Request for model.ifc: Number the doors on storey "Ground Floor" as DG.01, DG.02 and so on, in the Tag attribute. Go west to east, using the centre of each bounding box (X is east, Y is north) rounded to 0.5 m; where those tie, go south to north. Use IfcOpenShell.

First a look at what the model holds.

```python
import ifcopenshell
import ifcopenshell.util.element
import ifcopenshell.util.placement

model = ifcopenshell.open("model.ifc")
print(model.schema)
storey = next(s for s in model.by_type("IfcBuildingStorey") if s.Name == "Ground Floor")
doors = [e for e in ifcopenshell.util.element.get_decomposition(storey) if e.is_a("IfcDoor")]
for e in sorted(doors, key=lambda e: e.id()):
    origin = ifcopenshell.util.placement.get_local_placement(e.ObjectPlacement)[:3, 3]
    print(e.id(), e.Tag, e.Name, origin.round(2) + 0.0, sep=" | ")
```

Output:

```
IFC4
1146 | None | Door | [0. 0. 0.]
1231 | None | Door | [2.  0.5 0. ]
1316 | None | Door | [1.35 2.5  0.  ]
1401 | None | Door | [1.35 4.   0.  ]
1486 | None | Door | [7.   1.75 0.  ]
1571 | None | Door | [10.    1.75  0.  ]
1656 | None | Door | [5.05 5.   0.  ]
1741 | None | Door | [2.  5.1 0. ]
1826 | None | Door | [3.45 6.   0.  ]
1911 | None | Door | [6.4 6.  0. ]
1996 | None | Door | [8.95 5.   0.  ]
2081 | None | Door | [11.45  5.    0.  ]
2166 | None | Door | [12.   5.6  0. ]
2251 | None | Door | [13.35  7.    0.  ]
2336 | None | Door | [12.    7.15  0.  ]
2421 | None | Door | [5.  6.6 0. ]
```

```python
import ifcopenshell
import ifcopenshell.geom
import ifcopenshell.util.element
import ifcopenshell.util.shape

model = ifcopenshell.open("model.ifc")
settings = ifcopenshell.geom.settings()
settings.set("use-world-coords", True)


def centre(element):
    shape = ifcopenshell.geom.create_shape(settings, element)
    return ifcopenshell.util.shape.get_bbox_centroid(shape.geometry)


storey = next(s for s in model.by_type("IfcBuildingStorey") if s.Name == "Ground Floor")
doors = [e for e in ifcopenshell.util.element.get_decomposition(storey) if e.is_a("IfcDoor")]

# Insertion points can sit at a corner or the storey origin, so sort by the geometry (in metres).
centres = {e: centre(e) for e in doors}
doors.sort(key=lambda e: (round(centres[e][0] / 0.5), centres[e][1]))

for i, e in enumerate(doors, start=1):
    number = f"DG.{i:02d}"
    e.Tag = number
    print(e.id(), number)

model.write("model_v2.ifc")
```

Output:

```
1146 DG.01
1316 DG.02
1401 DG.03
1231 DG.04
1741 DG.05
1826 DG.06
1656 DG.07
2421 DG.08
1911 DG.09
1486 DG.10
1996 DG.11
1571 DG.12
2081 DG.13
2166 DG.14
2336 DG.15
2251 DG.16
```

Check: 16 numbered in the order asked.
